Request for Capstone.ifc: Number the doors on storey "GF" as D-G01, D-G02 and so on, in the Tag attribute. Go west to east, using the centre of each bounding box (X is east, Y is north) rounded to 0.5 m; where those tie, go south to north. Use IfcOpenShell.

First a look at what the model holds.

```python
import ifcopenshell
import ifcopenshell.util.element
import ifcopenshell.util.placement

model = ifcopenshell.open("Capstone.ifc")
print(model.schema)
storey = next(s for s in model.by_type("IfcBuildingStorey") if s.Name == "GF")
doors = [e for e in ifcopenshell.util.element.get_decomposition(storey) if e.is_a("IfcDoor")]
for e in sorted(doors, key=lambda e: e.id()):
    origin = ifcopenshell.util.placement.get_local_placement(e.ObjectPlacement)[:3, 3]
    print(e.id(), e.Tag, e.Name, origin.round(2) + 0.0, sep=" | ")
```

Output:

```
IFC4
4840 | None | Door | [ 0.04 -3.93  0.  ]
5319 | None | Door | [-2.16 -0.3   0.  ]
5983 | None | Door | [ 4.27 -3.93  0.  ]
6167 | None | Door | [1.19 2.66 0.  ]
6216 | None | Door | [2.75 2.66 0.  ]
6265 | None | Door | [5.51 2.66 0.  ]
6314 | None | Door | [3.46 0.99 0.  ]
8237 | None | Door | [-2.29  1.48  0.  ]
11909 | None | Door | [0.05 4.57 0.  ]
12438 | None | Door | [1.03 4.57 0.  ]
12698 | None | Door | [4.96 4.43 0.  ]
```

```python
import ifcopenshell
import ifcopenshell.geom
import ifcopenshell.util.element
import ifcopenshell.util.shape

model = ifcopenshell.open("Capstone.ifc")
settings = ifcopenshell.geom.settings()
settings.set("use-world-coords", True)


def centre(element):
    shape = ifcopenshell.geom.create_shape(settings, element)
    return ifcopenshell.util.shape.get_bbox_centroid(shape.geometry)


storey = next(s for s in model.by_type("IfcBuildingStorey") if s.Name == "GF")
doors = [e for e in ifcopenshell.util.element.get_decomposition(storey) if e.is_a("IfcDoor")]

# Insertion points can sit at a corner or the storey origin, so sort by the geometry (in metres).
centres = {e: centre(e) for e in doors}
doors.sort(key=lambda e: (round(centres[e][0] / 0.5), centres[e][1]))

for i, e in enumerate(doors, start=1):
    number = f"D-G{i:02d}"
    e.Tag = number
    print(e.id(), number)

model.write("Capstone_edited.ifc")
```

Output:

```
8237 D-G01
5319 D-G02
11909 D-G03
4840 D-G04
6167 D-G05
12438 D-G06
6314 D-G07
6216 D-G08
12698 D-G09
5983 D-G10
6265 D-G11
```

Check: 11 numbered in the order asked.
